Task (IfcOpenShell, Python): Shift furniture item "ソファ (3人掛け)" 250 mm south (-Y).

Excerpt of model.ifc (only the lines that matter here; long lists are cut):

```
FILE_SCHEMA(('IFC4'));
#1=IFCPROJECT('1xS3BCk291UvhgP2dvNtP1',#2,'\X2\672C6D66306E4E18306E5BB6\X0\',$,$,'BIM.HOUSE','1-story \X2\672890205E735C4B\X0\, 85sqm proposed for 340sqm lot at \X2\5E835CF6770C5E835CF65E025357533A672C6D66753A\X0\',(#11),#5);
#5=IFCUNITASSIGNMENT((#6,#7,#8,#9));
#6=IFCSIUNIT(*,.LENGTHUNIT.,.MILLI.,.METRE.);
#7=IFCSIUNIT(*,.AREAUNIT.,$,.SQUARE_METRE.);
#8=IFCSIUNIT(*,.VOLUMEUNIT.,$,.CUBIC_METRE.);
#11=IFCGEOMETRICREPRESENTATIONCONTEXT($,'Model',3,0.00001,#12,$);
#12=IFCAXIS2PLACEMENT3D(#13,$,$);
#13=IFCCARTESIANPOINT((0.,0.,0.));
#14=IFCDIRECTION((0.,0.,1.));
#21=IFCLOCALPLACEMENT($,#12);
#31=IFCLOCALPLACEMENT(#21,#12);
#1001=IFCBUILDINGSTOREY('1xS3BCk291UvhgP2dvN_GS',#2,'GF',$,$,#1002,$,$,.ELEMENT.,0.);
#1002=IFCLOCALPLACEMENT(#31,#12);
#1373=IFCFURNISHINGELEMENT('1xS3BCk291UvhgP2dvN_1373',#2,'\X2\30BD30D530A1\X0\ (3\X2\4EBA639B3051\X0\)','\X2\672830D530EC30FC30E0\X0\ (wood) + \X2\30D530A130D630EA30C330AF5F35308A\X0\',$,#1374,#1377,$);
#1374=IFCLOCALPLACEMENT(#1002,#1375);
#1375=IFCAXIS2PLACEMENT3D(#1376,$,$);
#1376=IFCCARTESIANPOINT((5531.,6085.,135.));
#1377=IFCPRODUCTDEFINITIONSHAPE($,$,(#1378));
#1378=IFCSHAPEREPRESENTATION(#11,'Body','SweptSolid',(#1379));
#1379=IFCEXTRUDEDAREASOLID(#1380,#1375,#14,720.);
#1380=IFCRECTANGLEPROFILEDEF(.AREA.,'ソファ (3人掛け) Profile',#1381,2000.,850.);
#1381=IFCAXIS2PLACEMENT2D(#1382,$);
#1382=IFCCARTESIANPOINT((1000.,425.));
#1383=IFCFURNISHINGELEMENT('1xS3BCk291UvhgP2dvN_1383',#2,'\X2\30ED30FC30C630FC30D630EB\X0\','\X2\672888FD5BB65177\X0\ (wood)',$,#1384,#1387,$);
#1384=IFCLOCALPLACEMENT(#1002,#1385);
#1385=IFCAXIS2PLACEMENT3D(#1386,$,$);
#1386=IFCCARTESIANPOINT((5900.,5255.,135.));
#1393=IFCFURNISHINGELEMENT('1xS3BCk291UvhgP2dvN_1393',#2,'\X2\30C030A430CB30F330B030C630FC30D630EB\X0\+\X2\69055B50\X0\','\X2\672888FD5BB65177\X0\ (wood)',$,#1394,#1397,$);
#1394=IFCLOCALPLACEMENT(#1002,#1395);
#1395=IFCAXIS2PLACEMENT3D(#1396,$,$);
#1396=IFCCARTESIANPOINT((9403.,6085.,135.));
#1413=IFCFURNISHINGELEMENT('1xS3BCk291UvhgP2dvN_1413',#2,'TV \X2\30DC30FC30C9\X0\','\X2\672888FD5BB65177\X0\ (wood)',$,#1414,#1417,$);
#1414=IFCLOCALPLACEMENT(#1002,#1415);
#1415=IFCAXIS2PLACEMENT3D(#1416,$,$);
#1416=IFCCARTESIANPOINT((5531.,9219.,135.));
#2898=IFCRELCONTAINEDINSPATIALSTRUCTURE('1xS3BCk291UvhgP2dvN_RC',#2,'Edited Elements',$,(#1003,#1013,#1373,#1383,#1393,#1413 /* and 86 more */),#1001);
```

```python
import ifcopenshell
import ifcopenshell.api.geometry
import ifcopenshell.util.placement
import ifcopenshell.util.unit

model = ifcopenshell.open("model.ifc")
unit_scale = ifcopenshell.util.unit.calculate_unit_scale(model)

item = model.by_guid("1xS3BCk291UvhgP2dvN_1373")
matrix = ifcopenshell.util.placement.get_local_placement(item.ObjectPlacement)
matrix[1, 3] -= 0.25 / unit_scale
ifcopenshell.api.geometry.edit_object_placement(model, product=item, matrix=matrix, is_si=False)

print(ifcopenshell.util.placement.get_local_placement(item.ObjectPlacement).round(3) + 0.0)

model.write("model_updated.ifc")
```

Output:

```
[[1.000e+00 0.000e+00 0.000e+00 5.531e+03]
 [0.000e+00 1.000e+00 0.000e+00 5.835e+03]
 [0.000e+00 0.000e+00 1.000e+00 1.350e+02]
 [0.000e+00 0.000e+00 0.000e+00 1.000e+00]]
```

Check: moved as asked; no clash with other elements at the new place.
